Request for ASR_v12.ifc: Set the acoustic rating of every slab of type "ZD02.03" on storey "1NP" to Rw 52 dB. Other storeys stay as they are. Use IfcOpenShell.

First a look at what the model holds.

```python
import ifcopenshell
import ifcopenshell.util.element

model = ifcopenshell.open("ASR_v12.ifc")
print(model.schema)
storey = next(s for s in model.by_type("IfcBuildingStorey") if s.Name == "1NP")
slabs = [e for e in ifcopenshell.util.element.get_decomposition(storey) if e.is_a("IfcSlab")]
seen = {}
for e in slabs:
    element_type = ifcopenshell.util.element.get_type(e)
    key = (element_type.Name if element_type != e and element_type else None, ifcopenshell.util.element.get_pset(e, "Pset_SlabCommon", "AcousticRating"))
    seen[key] = seen.get(key, 0) + 1
for (name, value), count in sorted(seen.items(), key=str):
    print(count, "x", name, "|", value)
```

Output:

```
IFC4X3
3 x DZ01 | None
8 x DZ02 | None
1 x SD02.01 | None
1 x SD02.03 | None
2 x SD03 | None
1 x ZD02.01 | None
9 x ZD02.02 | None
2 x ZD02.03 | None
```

```python
import ifcopenshell
import ifcopenshell.api.pset
import ifcopenshell.util.element

model = ifcopenshell.open("ASR_v12.ifc")

storey = next(s for s in model.by_type("IfcBuildingStorey") if s.Name == "1NP")
slabs = [e for e in ifcopenshell.util.element.get_decomposition(storey) if e.is_a("IfcSlab")]

count = 0
for e in slabs:
    element_type = ifcopenshell.util.element.get_type(e)
    if element_type in (None, e) or element_type.Name != "ZD02.03":
        continue
    # add_pset returns the element's existing set when there is one.
    pset = ifcopenshell.api.pset.add_pset(model, product=e, name="Pset_SlabCommon")
    ifcopenshell.api.pset.edit_pset(model, pset=pset, properties={"AcousticRating": "Rw 52 dB"})
    count += 1

print(count, "slabs updated")

model.write("ASR_v12_edited.ifc")
```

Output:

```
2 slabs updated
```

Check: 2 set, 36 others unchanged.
